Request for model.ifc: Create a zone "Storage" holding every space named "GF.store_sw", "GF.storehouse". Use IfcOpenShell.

First a look at what the model holds.

```python
import ifcopenshell

model = ifcopenshell.open("model.ifc")
print(model.schema)
seen = {}
for space in model.by_type("IfcSpace"):
    seen[space.LongName] = seen.get(space.LongName, 0) + 1
for name, count in sorted(seen.items(), key=str):
    print(count, "x", name)
print("zones:", [z.Name for z in model.by_type("IfcZone")][:20])
```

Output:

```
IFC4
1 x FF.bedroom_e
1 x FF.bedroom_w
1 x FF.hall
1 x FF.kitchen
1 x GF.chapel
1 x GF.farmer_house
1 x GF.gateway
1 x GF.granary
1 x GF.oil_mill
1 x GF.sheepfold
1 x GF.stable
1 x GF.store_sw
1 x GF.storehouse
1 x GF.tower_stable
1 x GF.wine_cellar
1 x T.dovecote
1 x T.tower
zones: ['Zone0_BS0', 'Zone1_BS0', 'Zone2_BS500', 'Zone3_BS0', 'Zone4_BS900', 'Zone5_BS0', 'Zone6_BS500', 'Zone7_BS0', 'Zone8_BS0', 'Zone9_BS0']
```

```python
import ifcopenshell
import ifcopenshell.api.group
import ifcopenshell.api.root

model = ifcopenshell.open("model.ifc")

names = {"GF.store_sw", "GF.storehouse"}
spaces = [s for s in model.by_type("IfcSpace") if s.LongName in names]

zone = ifcopenshell.api.root.create_entity(model, ifc_class="IfcZone", name="Storage")
ifcopenshell.api.group.assign_group(model, products=spaces, group=zone)
print(len(spaces), "spaces in", zone.Name)

model.write("model_edited.ifc")
```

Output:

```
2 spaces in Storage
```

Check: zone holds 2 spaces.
